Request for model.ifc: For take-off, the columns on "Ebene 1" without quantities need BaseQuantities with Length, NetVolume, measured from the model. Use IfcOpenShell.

First a look at what the model holds.

```python
import ifcopenshell
import ifcopenshell.util.element
import ifcopenshell.util.unit

model = ifcopenshell.open("model.ifc")
print(model.schema)
for unit_type in ("LENGTHUNIT", "AREAUNIT", "VOLUMEUNIT"):
    print(unit_type, ifcopenshell.util.unit.calculate_unit_scale(model, unit_type))
storey = next(s for s in model.by_type("IfcBuildingStorey") if s.Name == "Ebene 1")
columns = [e for e in ifcopenshell.util.element.get_decomposition(storey) if e.is_a("IfcColumn")]
for e in sorted(columns, key=lambda e: e.id()):
    print(e.id(), e.is_a(), e.Name, list(ifcopenshell.util.element.get_psets(e, qtos_only=True)), sep=" | ")
```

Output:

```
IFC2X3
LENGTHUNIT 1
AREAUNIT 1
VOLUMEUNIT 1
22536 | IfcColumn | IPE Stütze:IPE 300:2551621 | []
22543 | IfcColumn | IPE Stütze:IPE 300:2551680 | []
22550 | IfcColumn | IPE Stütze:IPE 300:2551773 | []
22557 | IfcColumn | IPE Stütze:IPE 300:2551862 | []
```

```python
import ifcopenshell
import ifcopenshell.api.pset
import ifcopenshell.geom
import ifcopenshell.util.element
import ifcopenshell.util.shape
import ifcopenshell.util.unit

model = ifcopenshell.open("model.ifc")
unit_scale = ifcopenshell.util.unit.calculate_unit_scale(model)
volume_scale = ifcopenshell.util.unit.calculate_unit_scale(model, "VOLUMEUNIT")
settings = ifcopenshell.geom.settings()

storey = next(s for s in model.by_type("IfcBuildingStorey") if s.Name == "Ebene 1")
columns = [e for e in ifcopenshell.util.element.get_decomposition(storey) if e.is_a("IfcColumn")]

for e in sorted(columns, key=lambda e: e.id()):
    if ifcopenshell.util.element.get_psets(e, qtos_only=True, should_inherit=False):
        continue
    # Geometry comes back in metres, in the element's own axes.
    shape = ifcopenshell.geom.create_shape(settings, e)
    values = {
        "Length": ifcopenshell.util.shape.get_z(shape.geometry) / unit_scale,
        "NetVolume": ifcopenshell.util.shape.get_volume(shape.geometry) / volume_scale,
    }
    qto = ifcopenshell.api.pset.add_qto(model, product=e, name="BaseQuantities")
    ifcopenshell.api.pset.edit_qto(model, qto=qto, properties=values)
    print(e.id(), {k: round(v, 3) for k, v in values.items()})

model.write("model_updated.ifc")
```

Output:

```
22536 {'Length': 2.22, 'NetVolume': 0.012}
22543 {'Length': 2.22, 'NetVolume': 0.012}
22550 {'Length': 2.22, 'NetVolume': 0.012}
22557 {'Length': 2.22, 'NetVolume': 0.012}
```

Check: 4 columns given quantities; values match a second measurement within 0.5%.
